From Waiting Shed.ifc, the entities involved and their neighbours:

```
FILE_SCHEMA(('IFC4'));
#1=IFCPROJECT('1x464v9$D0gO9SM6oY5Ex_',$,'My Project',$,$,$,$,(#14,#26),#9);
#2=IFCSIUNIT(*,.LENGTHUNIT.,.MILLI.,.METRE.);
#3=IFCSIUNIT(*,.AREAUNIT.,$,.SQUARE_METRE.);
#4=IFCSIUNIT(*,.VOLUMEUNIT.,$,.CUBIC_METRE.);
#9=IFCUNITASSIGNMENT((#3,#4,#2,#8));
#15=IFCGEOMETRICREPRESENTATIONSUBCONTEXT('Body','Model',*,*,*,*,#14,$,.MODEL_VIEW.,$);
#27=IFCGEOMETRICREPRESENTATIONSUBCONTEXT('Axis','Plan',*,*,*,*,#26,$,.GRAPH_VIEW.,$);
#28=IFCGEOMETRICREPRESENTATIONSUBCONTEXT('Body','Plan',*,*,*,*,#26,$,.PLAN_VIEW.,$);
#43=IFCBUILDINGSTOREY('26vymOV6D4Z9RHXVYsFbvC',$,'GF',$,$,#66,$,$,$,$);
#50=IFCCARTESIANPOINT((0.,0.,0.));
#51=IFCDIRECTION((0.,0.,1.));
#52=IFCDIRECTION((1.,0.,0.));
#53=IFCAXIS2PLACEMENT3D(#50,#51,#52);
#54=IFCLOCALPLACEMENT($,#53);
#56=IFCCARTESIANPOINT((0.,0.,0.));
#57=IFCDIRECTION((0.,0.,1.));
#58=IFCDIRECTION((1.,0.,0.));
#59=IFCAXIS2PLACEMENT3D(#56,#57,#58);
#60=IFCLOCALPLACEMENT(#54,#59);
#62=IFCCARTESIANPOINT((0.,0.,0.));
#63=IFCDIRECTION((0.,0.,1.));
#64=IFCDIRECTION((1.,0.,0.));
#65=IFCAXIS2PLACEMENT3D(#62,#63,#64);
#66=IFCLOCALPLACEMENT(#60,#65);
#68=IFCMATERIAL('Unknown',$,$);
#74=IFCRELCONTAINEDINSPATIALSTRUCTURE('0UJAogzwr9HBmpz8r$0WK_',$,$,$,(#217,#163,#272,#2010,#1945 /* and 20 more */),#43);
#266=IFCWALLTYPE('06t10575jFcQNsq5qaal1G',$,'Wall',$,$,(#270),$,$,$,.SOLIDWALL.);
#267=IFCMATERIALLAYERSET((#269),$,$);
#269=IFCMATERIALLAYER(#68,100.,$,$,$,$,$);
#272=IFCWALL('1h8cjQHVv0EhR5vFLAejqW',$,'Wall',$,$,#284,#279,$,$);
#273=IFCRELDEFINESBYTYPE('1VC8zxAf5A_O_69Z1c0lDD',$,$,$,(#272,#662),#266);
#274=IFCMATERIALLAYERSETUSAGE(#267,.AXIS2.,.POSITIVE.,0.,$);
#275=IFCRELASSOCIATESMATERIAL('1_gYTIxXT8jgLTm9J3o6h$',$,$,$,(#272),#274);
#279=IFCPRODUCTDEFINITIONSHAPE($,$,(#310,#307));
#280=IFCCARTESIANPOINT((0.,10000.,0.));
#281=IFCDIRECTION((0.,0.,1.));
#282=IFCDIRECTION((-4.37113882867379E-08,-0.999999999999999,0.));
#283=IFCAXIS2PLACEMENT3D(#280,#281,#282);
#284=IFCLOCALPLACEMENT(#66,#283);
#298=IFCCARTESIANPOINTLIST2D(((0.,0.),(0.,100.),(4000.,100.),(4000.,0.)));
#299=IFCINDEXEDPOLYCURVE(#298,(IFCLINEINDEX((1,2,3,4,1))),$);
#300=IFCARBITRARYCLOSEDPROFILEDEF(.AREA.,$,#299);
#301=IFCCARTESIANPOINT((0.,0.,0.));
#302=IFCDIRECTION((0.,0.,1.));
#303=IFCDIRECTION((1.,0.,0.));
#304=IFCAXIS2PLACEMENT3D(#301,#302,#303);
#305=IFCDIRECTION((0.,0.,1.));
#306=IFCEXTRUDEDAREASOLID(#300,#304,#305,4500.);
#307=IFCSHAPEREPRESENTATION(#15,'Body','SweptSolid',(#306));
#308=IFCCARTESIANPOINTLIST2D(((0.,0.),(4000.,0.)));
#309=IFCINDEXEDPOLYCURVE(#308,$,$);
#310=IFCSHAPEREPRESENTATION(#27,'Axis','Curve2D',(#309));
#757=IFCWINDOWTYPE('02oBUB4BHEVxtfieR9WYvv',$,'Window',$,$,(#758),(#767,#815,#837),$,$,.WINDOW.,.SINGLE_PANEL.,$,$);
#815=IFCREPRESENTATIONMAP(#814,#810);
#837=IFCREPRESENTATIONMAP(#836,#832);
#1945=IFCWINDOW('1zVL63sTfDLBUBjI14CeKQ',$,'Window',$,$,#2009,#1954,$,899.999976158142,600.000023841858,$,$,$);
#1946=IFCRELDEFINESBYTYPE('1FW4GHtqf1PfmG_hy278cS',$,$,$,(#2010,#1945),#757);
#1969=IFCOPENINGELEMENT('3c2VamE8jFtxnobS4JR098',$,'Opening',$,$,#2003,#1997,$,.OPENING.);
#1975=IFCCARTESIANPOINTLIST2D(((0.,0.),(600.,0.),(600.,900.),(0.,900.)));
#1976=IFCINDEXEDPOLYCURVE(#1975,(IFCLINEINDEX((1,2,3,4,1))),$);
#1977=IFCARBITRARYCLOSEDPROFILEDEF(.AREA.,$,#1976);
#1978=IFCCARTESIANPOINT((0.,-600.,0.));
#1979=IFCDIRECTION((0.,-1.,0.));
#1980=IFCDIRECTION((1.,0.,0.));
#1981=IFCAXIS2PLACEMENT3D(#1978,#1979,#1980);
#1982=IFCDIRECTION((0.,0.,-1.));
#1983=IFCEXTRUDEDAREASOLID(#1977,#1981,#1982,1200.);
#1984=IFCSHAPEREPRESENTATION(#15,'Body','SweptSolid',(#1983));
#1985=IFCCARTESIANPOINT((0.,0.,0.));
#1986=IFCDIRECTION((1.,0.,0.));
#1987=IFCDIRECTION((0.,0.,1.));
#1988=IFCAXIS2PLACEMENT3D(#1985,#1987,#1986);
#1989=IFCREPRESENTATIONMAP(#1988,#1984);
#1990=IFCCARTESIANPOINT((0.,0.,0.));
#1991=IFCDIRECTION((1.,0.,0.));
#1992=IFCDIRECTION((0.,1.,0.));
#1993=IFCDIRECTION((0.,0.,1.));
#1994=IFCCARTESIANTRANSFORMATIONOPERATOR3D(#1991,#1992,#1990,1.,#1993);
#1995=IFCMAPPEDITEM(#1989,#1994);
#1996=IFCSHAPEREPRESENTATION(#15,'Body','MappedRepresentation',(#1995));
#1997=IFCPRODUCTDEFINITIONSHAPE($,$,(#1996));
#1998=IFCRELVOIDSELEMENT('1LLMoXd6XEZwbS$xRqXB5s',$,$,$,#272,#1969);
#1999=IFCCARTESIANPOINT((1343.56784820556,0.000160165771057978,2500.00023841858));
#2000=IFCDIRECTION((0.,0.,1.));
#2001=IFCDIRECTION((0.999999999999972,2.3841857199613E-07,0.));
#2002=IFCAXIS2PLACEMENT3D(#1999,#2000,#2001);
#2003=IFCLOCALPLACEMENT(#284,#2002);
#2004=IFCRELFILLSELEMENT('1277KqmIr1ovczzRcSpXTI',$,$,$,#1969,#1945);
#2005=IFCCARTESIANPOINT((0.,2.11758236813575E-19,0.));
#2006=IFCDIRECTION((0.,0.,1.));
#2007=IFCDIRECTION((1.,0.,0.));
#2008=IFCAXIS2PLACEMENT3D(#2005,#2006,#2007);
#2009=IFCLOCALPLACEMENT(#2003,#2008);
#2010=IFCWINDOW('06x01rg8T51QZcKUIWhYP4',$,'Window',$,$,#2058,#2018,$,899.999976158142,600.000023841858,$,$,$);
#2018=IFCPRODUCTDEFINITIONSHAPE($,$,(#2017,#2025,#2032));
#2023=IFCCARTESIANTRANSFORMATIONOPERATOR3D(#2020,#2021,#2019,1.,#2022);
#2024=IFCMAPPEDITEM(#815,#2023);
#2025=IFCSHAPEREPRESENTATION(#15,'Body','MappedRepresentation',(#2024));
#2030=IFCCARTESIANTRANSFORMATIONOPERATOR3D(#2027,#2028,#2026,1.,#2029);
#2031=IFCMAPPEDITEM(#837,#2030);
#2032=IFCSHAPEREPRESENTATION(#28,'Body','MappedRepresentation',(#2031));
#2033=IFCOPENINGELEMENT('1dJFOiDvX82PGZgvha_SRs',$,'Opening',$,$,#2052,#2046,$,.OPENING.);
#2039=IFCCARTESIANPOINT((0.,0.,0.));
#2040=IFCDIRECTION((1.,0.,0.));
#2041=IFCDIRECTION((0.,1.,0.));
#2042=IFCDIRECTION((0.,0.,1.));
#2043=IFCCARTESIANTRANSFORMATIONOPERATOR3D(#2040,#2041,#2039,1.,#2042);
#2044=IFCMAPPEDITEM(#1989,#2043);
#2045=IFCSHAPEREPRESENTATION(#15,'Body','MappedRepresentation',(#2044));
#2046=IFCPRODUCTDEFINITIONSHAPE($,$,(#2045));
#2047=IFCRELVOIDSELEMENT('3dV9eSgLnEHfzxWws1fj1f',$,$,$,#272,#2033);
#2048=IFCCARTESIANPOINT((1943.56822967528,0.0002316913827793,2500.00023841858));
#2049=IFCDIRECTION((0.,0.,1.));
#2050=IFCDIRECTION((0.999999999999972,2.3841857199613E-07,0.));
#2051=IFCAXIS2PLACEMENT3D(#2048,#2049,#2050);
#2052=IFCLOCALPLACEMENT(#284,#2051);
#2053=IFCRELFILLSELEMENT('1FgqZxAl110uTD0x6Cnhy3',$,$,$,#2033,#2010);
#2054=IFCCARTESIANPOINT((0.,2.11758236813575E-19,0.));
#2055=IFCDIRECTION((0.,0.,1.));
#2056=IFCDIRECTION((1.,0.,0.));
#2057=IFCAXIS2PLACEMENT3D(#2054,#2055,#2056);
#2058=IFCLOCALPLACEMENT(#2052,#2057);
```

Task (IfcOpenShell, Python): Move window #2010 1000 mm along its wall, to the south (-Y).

```python
import ifcopenshell
import ifcopenshell.api.geometry
import ifcopenshell.util.placement

model = ifcopenshell.open("Waiting Shed.ifc")

window = model.by_id(2010)
opening = window.FillsVoids[0].RelatingOpeningElement
wall = opening.VoidsElements[0].RelatingBuildingElement

wall_matrix = ifcopenshell.util.placement.get_local_placement(wall.ObjectPlacement)
shift = wall_matrix[:3, 0] * 1000.0
before = ifcopenshell.util.placement.get_local_placement(window.ObjectPlacement)[:3, 3].copy()

# The window is placed relative to its opening, so it follows when the opening moves.
matrix = ifcopenshell.util.placement.get_local_placement(opening.ObjectPlacement)
matrix[:3, 3] += shift
ifcopenshell.api.geometry.edit_object_placement(
    model, product=opening, matrix=matrix, is_si=False, should_transform_children=True
)

after = ifcopenshell.util.placement.get_local_placement(window.ObjectPlacement)[:3, 3]
print("window moved by", (after - before).round(3) + 0.0)

model.write("Waiting Shed_edited.ifc")
```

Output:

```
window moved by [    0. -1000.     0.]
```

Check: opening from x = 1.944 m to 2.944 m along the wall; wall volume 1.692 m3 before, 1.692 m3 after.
